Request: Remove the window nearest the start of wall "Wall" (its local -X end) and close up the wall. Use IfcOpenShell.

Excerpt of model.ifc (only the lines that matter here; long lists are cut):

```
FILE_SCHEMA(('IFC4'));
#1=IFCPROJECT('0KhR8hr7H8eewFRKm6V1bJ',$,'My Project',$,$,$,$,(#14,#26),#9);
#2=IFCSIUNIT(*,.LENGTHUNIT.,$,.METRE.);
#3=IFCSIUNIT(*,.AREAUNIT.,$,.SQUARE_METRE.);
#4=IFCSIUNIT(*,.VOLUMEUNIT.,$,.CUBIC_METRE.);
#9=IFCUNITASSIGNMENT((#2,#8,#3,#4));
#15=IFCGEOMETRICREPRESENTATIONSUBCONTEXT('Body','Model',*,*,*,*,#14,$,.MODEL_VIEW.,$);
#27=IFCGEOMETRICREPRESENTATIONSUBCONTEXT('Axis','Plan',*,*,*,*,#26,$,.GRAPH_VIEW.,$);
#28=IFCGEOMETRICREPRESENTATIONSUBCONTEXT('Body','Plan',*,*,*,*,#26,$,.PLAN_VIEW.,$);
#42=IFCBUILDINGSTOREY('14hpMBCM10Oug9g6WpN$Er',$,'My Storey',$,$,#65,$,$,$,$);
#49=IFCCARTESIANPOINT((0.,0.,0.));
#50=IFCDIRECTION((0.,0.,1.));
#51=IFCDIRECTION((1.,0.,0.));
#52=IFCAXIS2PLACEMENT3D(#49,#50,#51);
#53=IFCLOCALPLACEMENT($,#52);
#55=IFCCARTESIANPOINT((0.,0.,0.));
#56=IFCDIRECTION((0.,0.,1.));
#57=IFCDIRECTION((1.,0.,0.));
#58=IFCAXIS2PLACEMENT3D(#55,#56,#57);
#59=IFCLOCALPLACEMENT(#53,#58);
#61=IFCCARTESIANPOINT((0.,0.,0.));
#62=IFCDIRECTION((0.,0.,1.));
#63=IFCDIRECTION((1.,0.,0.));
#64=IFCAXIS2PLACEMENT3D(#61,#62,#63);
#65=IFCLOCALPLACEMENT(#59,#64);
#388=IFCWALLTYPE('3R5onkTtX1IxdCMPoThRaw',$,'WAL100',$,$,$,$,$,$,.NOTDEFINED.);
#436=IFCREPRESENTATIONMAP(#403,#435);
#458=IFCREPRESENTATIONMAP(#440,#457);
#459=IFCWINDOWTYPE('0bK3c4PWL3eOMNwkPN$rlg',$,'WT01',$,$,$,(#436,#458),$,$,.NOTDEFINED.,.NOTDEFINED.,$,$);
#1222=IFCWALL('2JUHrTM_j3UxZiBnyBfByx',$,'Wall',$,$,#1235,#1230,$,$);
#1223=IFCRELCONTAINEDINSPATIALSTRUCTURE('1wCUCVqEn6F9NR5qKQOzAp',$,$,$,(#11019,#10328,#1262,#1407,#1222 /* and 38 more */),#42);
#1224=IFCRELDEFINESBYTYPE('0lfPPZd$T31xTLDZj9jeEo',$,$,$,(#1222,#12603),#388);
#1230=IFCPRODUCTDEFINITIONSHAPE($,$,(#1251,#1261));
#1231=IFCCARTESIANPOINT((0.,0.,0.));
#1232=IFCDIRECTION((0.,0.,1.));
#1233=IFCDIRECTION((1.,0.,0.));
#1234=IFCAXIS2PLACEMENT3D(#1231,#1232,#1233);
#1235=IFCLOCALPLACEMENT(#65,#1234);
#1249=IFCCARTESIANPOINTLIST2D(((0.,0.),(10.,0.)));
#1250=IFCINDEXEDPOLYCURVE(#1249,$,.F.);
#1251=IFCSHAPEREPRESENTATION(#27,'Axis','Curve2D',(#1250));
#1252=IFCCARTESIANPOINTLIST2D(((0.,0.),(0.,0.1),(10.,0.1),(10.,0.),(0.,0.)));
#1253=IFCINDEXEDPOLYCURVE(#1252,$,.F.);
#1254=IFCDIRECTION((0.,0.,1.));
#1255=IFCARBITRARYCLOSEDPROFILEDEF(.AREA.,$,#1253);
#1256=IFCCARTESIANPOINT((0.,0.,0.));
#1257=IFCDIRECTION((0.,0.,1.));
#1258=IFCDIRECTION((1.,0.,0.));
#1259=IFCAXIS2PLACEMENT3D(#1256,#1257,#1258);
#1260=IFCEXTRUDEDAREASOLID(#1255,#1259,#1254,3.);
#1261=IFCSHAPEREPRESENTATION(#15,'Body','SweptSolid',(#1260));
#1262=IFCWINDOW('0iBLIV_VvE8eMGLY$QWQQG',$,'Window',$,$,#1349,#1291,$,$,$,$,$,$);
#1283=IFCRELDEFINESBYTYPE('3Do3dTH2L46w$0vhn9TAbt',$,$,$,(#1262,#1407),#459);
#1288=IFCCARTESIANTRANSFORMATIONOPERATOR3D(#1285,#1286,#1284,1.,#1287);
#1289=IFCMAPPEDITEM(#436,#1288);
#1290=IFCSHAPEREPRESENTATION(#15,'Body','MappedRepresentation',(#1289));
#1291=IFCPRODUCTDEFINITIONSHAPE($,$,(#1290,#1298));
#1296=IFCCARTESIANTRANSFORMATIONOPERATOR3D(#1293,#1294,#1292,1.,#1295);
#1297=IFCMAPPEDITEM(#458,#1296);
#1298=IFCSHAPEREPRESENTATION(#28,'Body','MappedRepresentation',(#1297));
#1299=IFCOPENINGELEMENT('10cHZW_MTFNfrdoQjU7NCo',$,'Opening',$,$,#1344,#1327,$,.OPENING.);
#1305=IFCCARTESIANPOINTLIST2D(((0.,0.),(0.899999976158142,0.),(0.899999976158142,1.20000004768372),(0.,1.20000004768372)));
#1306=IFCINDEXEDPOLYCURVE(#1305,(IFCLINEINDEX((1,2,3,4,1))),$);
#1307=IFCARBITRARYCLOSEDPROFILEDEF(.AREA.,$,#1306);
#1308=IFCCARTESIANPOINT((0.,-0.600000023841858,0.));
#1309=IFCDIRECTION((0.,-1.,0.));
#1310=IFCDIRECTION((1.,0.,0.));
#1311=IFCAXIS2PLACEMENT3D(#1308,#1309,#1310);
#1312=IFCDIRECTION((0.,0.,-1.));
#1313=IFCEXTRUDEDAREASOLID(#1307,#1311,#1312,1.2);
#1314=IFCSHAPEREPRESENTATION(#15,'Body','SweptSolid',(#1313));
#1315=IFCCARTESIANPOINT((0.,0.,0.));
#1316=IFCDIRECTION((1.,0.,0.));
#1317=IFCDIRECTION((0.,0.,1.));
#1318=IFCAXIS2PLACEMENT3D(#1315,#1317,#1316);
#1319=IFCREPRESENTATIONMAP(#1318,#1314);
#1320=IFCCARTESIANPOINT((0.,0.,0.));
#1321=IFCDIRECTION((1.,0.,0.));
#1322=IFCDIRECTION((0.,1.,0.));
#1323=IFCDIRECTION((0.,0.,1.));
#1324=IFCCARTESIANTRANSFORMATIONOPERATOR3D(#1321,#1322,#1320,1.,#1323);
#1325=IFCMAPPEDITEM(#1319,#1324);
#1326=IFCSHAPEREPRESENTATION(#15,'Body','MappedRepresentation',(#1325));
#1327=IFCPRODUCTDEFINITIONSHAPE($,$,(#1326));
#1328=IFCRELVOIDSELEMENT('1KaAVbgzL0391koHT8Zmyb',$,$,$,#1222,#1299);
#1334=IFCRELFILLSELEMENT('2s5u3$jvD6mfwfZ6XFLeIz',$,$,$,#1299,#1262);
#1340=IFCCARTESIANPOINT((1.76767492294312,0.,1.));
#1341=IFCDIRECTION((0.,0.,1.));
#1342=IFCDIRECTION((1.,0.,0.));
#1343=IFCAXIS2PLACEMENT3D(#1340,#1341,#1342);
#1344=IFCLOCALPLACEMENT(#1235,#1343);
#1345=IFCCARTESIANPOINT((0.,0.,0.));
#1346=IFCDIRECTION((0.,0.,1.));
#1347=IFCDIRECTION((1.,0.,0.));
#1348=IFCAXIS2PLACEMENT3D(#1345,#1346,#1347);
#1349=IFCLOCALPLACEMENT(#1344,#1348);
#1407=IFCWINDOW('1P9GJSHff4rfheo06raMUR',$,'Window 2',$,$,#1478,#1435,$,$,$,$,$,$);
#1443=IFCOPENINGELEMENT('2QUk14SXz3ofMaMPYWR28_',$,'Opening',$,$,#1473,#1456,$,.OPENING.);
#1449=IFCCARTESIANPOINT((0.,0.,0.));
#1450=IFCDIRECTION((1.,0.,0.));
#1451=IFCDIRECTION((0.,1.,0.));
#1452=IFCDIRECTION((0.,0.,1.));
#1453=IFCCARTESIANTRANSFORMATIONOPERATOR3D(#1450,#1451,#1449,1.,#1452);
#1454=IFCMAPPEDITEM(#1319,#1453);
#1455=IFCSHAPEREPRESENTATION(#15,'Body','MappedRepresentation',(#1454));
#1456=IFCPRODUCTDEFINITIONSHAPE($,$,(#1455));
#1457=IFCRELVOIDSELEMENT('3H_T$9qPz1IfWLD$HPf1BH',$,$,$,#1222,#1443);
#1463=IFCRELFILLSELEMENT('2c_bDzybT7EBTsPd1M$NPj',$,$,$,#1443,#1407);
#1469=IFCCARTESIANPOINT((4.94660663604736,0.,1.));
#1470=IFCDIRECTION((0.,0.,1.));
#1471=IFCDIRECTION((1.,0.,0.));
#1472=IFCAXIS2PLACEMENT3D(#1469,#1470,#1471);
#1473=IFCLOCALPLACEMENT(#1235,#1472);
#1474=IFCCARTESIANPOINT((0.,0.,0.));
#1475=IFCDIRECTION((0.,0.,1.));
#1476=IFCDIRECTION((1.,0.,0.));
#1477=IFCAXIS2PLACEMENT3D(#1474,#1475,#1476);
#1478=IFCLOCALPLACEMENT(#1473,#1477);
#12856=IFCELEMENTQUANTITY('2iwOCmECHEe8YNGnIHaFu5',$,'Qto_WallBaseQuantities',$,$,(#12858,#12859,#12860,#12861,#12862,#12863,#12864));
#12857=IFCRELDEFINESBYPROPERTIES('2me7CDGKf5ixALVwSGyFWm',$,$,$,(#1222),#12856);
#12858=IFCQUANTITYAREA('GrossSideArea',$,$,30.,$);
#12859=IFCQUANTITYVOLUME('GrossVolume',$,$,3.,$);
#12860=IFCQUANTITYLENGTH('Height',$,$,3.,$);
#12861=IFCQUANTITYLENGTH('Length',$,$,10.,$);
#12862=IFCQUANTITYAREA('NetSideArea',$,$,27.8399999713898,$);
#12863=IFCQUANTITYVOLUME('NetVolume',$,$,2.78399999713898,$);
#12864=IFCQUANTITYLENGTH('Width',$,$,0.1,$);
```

```python
import ifcopenshell
import ifcopenshell.api.feature
import ifcopenshell.api.pset
import ifcopenshell.api.root
import ifcopenshell.geom
import ifcopenshell.util.element
import ifcopenshell.util.shape
import ifcopenshell.util.unit

model = ifcopenshell.open("model.ifc")
area_scale = ifcopenshell.util.unit.calculate_unit_scale(model, "AREAUNIT")
volume_scale = ifcopenshell.util.unit.calculate_unit_scale(model, "VOLUMEUNIT")
settings = ifcopenshell.geom.settings()


def volume(element):
    """Net volume in cubic metres, openings subtracted."""
    shape = ifcopenshell.geom.create_shape(settings, element)
    return ifcopenshell.util.shape.get_volume(shape.geometry)


window = model.by_guid("0iBLIV_VvE8eMGLY$QWQQG")
opening = window.FillsVoids[0].RelatingOpeningElement
wall = opening.VoidsElements[0].RelatingBuildingElement
before = volume(wall)

ifcopenshell.api.root.remove_product(model, product=window)
ifcopenshell.api.feature.remove_feature(model, feature=opening)

after = volume(wall)
thickness = 0.1  # wall thickness in metres

# Update the wall's stored quantities.
qto = model.by_id(ifcopenshell.util.element.get_pset(wall, "Qto_WallBaseQuantities", should_inherit=False)["id"])
ifcopenshell.api.pset.edit_qto(model, qto=qto, properties={
    "NetSideArea": after / thickness / area_scale,
    "NetVolume": after / volume_scale,
})

print(f"wall volume {before:.3f} -> {after:.3f} m3")

model.write("model_updated.ifc")
```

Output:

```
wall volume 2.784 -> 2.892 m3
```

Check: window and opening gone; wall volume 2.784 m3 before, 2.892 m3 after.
